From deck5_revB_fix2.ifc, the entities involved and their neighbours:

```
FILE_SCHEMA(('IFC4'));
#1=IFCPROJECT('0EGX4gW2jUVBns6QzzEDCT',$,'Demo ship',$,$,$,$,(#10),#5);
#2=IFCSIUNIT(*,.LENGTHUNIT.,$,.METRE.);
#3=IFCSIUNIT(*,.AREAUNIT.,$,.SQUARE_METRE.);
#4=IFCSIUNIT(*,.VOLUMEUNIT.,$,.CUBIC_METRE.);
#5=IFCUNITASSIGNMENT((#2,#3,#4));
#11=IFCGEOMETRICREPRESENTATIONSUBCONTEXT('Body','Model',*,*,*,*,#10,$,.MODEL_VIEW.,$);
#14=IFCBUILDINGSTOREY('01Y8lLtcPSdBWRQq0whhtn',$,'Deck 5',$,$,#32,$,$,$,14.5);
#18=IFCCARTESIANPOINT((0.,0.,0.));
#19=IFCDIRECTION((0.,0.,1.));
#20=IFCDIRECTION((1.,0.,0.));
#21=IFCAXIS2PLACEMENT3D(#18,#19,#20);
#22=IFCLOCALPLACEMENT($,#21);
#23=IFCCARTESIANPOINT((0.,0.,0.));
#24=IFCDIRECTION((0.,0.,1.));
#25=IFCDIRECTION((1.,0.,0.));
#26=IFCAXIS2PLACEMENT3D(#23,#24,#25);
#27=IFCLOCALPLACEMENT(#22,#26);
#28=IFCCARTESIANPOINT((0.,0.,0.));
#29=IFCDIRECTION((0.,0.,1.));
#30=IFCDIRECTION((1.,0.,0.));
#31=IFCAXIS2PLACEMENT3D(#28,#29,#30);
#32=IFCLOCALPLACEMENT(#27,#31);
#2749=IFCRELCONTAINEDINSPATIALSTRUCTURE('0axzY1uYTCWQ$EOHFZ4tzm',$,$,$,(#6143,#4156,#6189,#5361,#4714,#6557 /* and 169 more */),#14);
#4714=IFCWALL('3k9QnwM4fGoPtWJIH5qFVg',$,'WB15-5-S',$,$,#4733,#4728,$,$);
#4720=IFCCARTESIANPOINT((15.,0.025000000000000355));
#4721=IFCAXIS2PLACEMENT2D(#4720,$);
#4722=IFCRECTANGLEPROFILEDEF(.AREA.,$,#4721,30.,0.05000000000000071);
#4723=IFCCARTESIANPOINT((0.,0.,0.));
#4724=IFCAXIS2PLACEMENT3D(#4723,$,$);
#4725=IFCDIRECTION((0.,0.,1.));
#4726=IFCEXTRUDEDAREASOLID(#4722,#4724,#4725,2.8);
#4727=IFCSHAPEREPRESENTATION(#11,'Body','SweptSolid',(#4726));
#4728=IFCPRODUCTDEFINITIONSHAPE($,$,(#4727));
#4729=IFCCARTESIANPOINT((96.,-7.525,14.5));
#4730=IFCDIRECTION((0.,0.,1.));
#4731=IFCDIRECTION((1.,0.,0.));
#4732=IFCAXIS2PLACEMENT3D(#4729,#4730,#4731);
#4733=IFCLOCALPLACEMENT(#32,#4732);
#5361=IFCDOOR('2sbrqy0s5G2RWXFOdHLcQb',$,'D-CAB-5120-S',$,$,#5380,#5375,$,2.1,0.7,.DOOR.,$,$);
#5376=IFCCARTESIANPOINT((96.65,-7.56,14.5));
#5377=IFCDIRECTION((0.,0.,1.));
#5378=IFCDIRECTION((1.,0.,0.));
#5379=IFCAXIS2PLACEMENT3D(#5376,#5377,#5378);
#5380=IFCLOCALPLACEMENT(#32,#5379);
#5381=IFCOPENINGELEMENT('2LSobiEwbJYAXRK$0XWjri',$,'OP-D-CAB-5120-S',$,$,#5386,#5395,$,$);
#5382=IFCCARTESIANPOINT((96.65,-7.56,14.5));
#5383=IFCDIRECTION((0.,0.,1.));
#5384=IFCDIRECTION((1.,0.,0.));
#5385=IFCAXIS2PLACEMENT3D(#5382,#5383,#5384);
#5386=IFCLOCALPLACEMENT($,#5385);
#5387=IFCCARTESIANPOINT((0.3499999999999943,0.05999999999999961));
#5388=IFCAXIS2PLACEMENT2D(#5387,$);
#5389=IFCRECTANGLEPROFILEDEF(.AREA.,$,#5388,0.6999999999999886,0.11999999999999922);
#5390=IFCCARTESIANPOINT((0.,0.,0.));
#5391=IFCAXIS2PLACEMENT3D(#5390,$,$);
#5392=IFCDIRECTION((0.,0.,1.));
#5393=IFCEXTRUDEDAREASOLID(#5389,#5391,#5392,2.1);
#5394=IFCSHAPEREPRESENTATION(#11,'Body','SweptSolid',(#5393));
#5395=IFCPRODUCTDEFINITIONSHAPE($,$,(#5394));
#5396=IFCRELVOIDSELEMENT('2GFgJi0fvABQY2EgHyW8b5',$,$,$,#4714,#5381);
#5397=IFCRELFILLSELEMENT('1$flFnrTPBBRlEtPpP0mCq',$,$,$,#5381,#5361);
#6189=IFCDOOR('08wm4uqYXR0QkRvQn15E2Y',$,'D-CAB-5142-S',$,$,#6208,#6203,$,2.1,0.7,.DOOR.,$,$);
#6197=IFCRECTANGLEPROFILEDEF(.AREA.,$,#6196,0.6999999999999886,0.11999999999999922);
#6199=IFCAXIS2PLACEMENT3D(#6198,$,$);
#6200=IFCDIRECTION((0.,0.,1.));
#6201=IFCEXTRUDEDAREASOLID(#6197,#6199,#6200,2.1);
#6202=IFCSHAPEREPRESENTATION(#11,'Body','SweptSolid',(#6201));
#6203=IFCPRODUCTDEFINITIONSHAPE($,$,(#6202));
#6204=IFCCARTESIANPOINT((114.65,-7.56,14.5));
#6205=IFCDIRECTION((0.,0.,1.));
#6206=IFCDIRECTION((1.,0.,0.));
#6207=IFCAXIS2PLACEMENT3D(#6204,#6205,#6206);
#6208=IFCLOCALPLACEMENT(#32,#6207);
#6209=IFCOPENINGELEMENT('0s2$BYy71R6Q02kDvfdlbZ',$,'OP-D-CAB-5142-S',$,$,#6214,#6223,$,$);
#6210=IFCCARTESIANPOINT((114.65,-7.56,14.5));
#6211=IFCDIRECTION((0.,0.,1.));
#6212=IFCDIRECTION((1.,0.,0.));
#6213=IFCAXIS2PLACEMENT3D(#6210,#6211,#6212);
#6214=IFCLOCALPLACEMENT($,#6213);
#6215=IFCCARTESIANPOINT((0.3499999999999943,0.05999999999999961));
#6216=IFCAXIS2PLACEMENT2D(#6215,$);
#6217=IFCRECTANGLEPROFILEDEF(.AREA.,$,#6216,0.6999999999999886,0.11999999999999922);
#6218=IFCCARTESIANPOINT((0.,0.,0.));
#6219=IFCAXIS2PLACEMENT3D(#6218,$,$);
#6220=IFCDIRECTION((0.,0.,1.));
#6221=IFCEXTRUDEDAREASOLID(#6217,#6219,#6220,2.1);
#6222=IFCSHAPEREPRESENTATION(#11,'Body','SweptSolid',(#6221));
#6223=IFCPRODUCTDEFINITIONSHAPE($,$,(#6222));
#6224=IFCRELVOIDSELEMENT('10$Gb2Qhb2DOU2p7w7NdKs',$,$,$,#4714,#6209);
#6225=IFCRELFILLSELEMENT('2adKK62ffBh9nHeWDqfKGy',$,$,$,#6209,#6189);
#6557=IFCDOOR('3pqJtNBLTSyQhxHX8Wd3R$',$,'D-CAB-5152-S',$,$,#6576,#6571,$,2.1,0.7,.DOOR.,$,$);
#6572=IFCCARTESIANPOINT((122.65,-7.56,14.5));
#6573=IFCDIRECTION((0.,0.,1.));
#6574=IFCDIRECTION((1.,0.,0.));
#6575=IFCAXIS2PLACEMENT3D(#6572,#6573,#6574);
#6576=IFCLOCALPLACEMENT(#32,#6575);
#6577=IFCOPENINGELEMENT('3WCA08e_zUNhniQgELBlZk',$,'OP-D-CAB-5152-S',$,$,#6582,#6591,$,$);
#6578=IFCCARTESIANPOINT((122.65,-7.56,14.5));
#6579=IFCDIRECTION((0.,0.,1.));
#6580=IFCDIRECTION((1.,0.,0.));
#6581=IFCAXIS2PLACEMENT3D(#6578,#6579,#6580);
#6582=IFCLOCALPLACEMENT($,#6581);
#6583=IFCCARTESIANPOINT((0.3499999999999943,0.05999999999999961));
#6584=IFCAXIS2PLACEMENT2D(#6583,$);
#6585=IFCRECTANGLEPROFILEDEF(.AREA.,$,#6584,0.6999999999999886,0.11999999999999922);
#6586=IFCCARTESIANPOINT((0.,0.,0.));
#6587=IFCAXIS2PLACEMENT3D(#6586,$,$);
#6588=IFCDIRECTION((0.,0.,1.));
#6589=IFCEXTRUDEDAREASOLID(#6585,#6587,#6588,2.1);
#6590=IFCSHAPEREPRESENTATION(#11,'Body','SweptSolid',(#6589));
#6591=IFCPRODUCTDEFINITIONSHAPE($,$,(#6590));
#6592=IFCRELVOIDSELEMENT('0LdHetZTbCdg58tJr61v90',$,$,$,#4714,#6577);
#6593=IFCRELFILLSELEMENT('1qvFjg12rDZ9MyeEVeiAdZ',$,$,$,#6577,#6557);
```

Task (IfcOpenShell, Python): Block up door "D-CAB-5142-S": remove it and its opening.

```python
import ifcopenshell
import ifcopenshell.api.feature
import ifcopenshell.api.root
import ifcopenshell.geom
import ifcopenshell.util.shape

model = ifcopenshell.open("deck5_revB_fix2.ifc")
settings = ifcopenshell.geom.settings()


def volume(element):
    """Net volume in cubic metres, openings subtracted."""
    shape = ifcopenshell.geom.create_shape(settings, element)
    return ifcopenshell.util.shape.get_volume(shape.geometry)


door = model.by_guid("08wm4uqYXR0QkRvQn15E2Y")
opening = door.FillsVoids[0].RelatingOpeningElement
wall = opening.VoidsElements[0].RelatingBuildingElement
before = volume(wall)

ifcopenshell.api.root.remove_product(model, product=door)
ifcopenshell.api.feature.remove_feature(model, feature=opening)

after = volume(wall)

print(f"wall volume {before:.3f} -> {after:.3f} m3")

model.write("deck5_revB_fix2_rev.ifc")
```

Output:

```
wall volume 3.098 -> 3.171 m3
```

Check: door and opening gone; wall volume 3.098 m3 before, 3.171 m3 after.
